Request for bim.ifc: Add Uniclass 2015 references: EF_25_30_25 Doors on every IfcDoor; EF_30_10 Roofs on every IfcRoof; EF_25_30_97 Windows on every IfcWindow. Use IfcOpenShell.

First a look at what the model holds.

```python
import ifcopenshell

model = ifcopenshell.open("bim.ifc")
print(model.schema)
print("classifications:", [c.Name for c in model.by_type("IfcClassification")])
for ifc_class in ("IfcDoor", "IfcRoof", "IfcStair", "IfcWall", "IfcWindow"):
    print(ifc_class, len(model.by_type(ifc_class)))
```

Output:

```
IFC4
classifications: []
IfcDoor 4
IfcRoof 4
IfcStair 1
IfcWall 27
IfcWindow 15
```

```python
import ifcopenshell
import ifcopenshell.api.classification

model = ifcopenshell.open("bim.ifc")

system = ifcopenshell.api.classification.add_classification(model, classification="Uniclass 2015")

codes = {
    "IfcDoor": ("EF_25_30_25", "Doors"),
    "IfcRoof": ("EF_30_10", "Roofs"),
    "IfcWindow": ("EF_25_30_97", "Windows"),
}
for ifc_class, (code, name) in codes.items():
    products = model.by_type(ifc_class)
    ifcopenshell.api.classification.add_reference(
        model, products=products, classification=system, identification=code, name=name
    )
    print(code, len(products))

model.write("bim_rev.ifc")
```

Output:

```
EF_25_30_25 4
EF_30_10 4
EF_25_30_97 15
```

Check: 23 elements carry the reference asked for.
